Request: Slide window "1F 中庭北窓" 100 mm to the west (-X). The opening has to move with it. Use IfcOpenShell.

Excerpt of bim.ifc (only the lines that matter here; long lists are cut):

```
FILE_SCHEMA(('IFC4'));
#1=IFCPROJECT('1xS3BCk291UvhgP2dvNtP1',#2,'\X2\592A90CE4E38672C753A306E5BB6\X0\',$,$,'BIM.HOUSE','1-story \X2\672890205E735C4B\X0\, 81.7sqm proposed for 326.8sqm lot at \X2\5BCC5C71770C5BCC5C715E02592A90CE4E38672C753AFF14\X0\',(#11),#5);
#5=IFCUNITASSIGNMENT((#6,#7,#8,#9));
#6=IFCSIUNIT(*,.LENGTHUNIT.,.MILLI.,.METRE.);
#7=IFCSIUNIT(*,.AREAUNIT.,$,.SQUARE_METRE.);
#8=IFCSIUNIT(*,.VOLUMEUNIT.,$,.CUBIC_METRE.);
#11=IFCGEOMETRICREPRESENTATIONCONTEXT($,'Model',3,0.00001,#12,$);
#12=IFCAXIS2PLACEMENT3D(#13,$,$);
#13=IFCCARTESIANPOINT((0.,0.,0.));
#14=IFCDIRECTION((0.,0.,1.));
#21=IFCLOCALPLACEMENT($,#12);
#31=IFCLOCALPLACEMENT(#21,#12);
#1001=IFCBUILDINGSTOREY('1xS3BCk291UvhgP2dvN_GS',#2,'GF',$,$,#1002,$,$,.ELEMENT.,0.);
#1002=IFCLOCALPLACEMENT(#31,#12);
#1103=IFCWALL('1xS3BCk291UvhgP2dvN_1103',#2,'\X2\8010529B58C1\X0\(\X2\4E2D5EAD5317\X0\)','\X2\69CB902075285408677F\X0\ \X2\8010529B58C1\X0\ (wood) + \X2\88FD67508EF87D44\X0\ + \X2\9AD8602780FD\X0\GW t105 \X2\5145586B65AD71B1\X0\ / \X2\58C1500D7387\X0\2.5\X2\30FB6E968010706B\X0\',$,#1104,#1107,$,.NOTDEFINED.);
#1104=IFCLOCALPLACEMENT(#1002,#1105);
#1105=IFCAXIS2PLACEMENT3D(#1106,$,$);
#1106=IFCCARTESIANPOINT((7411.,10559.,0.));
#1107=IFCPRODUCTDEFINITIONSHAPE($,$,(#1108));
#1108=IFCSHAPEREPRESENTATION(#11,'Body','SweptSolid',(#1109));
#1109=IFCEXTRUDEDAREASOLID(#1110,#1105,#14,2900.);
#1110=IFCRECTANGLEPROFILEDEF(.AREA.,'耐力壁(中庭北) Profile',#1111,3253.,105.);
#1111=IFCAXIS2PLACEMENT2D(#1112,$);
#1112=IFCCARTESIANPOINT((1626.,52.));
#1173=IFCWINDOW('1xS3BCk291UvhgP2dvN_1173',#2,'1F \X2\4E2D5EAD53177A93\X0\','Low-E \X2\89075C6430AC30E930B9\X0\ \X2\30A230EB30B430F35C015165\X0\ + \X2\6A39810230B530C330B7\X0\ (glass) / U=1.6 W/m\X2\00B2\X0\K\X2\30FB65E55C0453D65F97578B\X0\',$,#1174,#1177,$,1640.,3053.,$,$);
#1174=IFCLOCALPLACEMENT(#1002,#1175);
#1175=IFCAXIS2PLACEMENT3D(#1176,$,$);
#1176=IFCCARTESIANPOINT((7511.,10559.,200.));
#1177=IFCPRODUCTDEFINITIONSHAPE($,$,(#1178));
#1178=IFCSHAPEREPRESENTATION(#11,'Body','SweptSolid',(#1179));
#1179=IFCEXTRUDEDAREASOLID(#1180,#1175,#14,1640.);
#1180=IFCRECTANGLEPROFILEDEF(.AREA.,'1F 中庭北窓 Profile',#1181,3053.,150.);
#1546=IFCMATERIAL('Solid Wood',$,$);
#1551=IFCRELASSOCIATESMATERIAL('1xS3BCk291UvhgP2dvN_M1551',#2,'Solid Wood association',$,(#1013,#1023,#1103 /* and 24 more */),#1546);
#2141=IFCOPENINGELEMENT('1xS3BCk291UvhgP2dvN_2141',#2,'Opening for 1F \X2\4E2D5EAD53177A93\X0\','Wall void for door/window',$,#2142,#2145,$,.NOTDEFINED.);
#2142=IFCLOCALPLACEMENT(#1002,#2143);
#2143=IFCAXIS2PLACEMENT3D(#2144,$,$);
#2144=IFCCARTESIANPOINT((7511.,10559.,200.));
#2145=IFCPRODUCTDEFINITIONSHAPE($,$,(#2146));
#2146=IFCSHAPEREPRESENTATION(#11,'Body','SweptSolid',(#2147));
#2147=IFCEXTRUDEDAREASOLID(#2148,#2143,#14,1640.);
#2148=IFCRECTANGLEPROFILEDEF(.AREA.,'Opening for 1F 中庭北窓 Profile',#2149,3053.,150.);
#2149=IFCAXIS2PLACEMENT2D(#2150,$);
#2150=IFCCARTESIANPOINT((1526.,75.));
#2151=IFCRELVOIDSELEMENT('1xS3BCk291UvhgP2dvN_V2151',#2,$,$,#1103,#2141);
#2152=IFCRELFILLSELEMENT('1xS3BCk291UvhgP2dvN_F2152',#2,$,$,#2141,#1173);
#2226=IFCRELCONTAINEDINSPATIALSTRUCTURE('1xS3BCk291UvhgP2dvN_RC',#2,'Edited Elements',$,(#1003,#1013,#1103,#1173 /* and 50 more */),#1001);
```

```python
import ifcopenshell
import ifcopenshell.api.geometry
import ifcopenshell.util.placement
import ifcopenshell.util.unit

model = ifcopenshell.open("bim.ifc")
unit_scale = ifcopenshell.util.unit.calculate_unit_scale(model)

window = model.by_id(1173)
opening = window.FillsVoids[0].RelatingOpeningElement
wall = opening.VoidsElements[0].RelatingBuildingElement

wall_matrix = ifcopenshell.util.placement.get_local_placement(wall.ObjectPlacement)
shift = wall_matrix[:3, 0] * -0.1 / unit_scale
before = ifcopenshell.util.placement.get_local_placement(window.ObjectPlacement)[:3, 3].copy()

# The window is not placed relative to its opening, so move both.
for product in (opening, window):
    matrix = ifcopenshell.util.placement.get_local_placement(product.ObjectPlacement)
    matrix[:3, 3] += shift
    ifcopenshell.api.geometry.edit_object_placement(model, product=product, matrix=matrix, is_si=False)

after = ifcopenshell.util.placement.get_local_placement(window.ObjectPlacement)[:3, 3]
print("window moved by", (after - before).round(3) + 0.0)

model.write("bim_edited.ifc")
```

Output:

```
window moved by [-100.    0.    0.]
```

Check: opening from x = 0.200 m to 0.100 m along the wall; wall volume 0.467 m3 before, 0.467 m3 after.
